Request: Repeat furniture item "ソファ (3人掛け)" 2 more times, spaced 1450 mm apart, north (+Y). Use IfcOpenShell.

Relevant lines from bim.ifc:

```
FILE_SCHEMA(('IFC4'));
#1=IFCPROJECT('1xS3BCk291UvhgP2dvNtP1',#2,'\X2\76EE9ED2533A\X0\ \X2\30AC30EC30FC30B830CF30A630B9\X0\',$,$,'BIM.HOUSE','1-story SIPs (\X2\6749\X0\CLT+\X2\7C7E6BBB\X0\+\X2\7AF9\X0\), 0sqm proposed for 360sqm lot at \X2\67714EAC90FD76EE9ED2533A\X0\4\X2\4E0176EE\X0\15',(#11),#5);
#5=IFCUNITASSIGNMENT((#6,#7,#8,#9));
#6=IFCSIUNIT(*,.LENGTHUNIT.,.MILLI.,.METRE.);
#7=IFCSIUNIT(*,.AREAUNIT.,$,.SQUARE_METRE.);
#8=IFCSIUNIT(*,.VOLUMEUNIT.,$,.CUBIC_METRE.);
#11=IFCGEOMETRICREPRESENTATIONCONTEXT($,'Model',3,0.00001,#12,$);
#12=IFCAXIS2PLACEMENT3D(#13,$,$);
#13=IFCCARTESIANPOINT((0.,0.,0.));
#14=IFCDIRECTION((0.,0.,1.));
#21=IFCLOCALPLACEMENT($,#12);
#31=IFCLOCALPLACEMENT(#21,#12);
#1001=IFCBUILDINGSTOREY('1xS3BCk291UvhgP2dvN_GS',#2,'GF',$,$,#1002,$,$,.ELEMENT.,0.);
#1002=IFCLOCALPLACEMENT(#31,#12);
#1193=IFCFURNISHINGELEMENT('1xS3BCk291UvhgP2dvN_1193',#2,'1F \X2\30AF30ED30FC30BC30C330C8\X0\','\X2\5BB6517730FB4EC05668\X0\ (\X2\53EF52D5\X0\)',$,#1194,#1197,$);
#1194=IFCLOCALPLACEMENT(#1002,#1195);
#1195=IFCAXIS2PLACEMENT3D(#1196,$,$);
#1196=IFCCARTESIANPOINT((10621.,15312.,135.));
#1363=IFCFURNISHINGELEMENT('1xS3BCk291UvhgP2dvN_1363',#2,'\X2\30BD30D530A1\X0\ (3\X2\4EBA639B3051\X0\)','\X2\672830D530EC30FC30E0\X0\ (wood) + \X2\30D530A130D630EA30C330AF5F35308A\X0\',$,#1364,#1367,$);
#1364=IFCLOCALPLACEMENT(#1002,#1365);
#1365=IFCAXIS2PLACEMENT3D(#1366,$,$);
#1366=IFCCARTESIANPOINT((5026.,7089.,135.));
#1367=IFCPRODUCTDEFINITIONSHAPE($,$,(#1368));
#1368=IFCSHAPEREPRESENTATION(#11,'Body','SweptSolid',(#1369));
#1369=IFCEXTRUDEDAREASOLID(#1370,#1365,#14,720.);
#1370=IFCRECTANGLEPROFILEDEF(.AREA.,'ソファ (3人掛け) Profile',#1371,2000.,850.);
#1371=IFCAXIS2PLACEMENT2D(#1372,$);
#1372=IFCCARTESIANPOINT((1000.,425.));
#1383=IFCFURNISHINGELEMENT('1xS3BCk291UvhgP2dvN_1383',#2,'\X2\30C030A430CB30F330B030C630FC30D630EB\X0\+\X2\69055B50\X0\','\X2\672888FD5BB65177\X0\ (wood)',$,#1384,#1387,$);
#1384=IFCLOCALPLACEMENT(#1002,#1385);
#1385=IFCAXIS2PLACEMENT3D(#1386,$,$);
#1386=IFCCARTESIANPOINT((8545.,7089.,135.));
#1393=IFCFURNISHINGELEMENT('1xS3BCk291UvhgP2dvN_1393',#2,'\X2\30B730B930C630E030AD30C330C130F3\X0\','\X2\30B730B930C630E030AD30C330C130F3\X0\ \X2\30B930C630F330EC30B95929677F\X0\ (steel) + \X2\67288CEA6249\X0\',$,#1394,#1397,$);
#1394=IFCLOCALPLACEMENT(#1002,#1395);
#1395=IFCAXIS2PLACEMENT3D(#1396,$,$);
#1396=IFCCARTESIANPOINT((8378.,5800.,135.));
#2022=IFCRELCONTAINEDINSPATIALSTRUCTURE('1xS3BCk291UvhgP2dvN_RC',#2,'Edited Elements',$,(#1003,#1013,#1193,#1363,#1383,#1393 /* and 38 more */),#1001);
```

```python
import numpy as np
import ifcopenshell
import ifcopenshell.api.geometry
import ifcopenshell.api.root
import ifcopenshell.util.element
import ifcopenshell.util.placement
import ifcopenshell.util.unit

model = ifcopenshell.open("bim.ifc")
unit_scale = ifcopenshell.util.unit.calculate_unit_scale(model)


def reuse_history(source, copy):
    """copy_class also copies each property set's owner history, people and application; keep the originals."""
    for rel in copy.IsDefinedBy:
        if rel.is_a("IfcRelDefinesByProperties") and (history := rel.RelatingPropertyDefinition.OwnerHistory):
            rel.RelatingPropertyDefinition.OwnerHistory = source.OwnerHistory
            ifcopenshell.util.element.remove_deep2(model, history)


source = model.by_id(1363)
base = ifcopenshell.util.placement.get_local_placement(source.ObjectPlacement)
step = np.array([0.0, 1.0, 0.0]) * 1.45 / unit_scale

for i in range(1, 3):
    copy = ifcopenshell.api.root.copy_class(model, product=source)
    copy.Representation = ifcopenshell.util.element.copy_deep(
        model, source.Representation, exclude=["IfcGeometricRepresentationContext", "IfcRepresentationMap"]
    )
    reuse_history(source, copy)
    matrix = base.copy()
    matrix[:3, 3] += i * step
    print("added at", matrix[:3, 3].round(3) + 0.0)
    ifcopenshell.api.geometry.edit_object_placement(model, product=copy, matrix=matrix, is_si=False)

model.write("bim_edited.ifc")
```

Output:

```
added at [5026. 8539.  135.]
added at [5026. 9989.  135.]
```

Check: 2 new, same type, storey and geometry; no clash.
